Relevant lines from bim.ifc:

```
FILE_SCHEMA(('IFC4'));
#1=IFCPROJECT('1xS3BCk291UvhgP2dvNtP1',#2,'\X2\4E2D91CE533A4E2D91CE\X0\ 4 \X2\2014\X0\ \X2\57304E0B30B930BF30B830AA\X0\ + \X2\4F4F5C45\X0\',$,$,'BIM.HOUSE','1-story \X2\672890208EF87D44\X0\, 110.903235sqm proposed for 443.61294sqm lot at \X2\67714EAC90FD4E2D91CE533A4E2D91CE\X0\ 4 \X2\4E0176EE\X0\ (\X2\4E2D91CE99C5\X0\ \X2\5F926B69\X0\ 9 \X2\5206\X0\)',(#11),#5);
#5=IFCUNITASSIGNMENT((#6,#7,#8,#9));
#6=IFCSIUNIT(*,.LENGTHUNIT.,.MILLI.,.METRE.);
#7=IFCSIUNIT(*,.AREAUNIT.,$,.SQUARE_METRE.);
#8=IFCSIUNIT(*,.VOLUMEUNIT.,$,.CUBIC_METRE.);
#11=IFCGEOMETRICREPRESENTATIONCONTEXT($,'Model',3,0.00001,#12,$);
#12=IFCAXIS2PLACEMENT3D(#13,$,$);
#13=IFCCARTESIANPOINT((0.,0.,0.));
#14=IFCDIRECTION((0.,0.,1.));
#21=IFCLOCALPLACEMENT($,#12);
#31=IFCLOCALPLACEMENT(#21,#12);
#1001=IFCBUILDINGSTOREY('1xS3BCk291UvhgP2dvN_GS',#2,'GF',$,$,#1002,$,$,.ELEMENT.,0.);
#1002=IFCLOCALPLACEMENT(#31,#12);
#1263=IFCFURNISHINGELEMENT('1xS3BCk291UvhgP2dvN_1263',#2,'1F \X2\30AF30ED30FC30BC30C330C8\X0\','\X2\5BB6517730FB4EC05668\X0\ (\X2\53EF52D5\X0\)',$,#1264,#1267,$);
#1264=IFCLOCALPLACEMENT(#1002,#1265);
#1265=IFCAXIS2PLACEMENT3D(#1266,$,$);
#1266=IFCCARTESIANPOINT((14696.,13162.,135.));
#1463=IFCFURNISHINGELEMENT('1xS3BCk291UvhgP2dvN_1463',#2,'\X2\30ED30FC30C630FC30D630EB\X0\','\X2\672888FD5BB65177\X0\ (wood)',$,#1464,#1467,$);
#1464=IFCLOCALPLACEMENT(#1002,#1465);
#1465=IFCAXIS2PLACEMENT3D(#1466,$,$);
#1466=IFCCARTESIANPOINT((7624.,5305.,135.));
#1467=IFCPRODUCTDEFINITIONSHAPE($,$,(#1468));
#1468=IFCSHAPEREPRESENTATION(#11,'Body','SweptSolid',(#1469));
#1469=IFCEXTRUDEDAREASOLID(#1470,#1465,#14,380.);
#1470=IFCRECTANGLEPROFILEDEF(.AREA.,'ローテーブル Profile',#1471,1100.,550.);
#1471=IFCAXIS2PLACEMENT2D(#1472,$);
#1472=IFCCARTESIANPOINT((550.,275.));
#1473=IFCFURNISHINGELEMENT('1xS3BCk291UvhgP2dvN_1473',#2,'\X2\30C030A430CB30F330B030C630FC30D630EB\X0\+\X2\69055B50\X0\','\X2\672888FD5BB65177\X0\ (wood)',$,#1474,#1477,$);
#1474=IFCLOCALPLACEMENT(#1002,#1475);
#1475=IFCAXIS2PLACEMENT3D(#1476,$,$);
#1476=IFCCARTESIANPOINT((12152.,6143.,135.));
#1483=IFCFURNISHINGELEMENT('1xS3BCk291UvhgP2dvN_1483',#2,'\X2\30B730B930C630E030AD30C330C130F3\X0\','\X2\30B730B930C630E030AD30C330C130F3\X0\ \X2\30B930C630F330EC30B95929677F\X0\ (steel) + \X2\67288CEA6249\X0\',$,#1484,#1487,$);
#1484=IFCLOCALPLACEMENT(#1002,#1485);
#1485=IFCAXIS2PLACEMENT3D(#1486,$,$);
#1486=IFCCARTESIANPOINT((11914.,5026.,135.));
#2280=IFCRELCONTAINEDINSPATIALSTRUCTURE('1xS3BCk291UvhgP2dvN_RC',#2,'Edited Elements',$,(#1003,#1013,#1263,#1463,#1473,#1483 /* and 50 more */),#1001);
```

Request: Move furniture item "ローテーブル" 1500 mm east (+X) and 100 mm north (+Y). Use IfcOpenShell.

```python
import ifcopenshell
import ifcopenshell.api.geometry
import ifcopenshell.util.placement
import ifcopenshell.util.unit

model = ifcopenshell.open("bim.ifc")
unit_scale = ifcopenshell.util.unit.calculate_unit_scale(model)

item = model.by_guid("1xS3BCk291UvhgP2dvN_1463")
matrix = ifcopenshell.util.placement.get_local_placement(item.ObjectPlacement)
matrix[0, 3] += 1.5 / unit_scale
matrix[1, 3] += 0.1 / unit_scale
ifcopenshell.api.geometry.edit_object_placement(model, product=item, matrix=matrix, is_si=False)

print(ifcopenshell.util.placement.get_local_placement(item.ObjectPlacement).round(3) + 0.0)

model.write("bim_rev.ifc")
```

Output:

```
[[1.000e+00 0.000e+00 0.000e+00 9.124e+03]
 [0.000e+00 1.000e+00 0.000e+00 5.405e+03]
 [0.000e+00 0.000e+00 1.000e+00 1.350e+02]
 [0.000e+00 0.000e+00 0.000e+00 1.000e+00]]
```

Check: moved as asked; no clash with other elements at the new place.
